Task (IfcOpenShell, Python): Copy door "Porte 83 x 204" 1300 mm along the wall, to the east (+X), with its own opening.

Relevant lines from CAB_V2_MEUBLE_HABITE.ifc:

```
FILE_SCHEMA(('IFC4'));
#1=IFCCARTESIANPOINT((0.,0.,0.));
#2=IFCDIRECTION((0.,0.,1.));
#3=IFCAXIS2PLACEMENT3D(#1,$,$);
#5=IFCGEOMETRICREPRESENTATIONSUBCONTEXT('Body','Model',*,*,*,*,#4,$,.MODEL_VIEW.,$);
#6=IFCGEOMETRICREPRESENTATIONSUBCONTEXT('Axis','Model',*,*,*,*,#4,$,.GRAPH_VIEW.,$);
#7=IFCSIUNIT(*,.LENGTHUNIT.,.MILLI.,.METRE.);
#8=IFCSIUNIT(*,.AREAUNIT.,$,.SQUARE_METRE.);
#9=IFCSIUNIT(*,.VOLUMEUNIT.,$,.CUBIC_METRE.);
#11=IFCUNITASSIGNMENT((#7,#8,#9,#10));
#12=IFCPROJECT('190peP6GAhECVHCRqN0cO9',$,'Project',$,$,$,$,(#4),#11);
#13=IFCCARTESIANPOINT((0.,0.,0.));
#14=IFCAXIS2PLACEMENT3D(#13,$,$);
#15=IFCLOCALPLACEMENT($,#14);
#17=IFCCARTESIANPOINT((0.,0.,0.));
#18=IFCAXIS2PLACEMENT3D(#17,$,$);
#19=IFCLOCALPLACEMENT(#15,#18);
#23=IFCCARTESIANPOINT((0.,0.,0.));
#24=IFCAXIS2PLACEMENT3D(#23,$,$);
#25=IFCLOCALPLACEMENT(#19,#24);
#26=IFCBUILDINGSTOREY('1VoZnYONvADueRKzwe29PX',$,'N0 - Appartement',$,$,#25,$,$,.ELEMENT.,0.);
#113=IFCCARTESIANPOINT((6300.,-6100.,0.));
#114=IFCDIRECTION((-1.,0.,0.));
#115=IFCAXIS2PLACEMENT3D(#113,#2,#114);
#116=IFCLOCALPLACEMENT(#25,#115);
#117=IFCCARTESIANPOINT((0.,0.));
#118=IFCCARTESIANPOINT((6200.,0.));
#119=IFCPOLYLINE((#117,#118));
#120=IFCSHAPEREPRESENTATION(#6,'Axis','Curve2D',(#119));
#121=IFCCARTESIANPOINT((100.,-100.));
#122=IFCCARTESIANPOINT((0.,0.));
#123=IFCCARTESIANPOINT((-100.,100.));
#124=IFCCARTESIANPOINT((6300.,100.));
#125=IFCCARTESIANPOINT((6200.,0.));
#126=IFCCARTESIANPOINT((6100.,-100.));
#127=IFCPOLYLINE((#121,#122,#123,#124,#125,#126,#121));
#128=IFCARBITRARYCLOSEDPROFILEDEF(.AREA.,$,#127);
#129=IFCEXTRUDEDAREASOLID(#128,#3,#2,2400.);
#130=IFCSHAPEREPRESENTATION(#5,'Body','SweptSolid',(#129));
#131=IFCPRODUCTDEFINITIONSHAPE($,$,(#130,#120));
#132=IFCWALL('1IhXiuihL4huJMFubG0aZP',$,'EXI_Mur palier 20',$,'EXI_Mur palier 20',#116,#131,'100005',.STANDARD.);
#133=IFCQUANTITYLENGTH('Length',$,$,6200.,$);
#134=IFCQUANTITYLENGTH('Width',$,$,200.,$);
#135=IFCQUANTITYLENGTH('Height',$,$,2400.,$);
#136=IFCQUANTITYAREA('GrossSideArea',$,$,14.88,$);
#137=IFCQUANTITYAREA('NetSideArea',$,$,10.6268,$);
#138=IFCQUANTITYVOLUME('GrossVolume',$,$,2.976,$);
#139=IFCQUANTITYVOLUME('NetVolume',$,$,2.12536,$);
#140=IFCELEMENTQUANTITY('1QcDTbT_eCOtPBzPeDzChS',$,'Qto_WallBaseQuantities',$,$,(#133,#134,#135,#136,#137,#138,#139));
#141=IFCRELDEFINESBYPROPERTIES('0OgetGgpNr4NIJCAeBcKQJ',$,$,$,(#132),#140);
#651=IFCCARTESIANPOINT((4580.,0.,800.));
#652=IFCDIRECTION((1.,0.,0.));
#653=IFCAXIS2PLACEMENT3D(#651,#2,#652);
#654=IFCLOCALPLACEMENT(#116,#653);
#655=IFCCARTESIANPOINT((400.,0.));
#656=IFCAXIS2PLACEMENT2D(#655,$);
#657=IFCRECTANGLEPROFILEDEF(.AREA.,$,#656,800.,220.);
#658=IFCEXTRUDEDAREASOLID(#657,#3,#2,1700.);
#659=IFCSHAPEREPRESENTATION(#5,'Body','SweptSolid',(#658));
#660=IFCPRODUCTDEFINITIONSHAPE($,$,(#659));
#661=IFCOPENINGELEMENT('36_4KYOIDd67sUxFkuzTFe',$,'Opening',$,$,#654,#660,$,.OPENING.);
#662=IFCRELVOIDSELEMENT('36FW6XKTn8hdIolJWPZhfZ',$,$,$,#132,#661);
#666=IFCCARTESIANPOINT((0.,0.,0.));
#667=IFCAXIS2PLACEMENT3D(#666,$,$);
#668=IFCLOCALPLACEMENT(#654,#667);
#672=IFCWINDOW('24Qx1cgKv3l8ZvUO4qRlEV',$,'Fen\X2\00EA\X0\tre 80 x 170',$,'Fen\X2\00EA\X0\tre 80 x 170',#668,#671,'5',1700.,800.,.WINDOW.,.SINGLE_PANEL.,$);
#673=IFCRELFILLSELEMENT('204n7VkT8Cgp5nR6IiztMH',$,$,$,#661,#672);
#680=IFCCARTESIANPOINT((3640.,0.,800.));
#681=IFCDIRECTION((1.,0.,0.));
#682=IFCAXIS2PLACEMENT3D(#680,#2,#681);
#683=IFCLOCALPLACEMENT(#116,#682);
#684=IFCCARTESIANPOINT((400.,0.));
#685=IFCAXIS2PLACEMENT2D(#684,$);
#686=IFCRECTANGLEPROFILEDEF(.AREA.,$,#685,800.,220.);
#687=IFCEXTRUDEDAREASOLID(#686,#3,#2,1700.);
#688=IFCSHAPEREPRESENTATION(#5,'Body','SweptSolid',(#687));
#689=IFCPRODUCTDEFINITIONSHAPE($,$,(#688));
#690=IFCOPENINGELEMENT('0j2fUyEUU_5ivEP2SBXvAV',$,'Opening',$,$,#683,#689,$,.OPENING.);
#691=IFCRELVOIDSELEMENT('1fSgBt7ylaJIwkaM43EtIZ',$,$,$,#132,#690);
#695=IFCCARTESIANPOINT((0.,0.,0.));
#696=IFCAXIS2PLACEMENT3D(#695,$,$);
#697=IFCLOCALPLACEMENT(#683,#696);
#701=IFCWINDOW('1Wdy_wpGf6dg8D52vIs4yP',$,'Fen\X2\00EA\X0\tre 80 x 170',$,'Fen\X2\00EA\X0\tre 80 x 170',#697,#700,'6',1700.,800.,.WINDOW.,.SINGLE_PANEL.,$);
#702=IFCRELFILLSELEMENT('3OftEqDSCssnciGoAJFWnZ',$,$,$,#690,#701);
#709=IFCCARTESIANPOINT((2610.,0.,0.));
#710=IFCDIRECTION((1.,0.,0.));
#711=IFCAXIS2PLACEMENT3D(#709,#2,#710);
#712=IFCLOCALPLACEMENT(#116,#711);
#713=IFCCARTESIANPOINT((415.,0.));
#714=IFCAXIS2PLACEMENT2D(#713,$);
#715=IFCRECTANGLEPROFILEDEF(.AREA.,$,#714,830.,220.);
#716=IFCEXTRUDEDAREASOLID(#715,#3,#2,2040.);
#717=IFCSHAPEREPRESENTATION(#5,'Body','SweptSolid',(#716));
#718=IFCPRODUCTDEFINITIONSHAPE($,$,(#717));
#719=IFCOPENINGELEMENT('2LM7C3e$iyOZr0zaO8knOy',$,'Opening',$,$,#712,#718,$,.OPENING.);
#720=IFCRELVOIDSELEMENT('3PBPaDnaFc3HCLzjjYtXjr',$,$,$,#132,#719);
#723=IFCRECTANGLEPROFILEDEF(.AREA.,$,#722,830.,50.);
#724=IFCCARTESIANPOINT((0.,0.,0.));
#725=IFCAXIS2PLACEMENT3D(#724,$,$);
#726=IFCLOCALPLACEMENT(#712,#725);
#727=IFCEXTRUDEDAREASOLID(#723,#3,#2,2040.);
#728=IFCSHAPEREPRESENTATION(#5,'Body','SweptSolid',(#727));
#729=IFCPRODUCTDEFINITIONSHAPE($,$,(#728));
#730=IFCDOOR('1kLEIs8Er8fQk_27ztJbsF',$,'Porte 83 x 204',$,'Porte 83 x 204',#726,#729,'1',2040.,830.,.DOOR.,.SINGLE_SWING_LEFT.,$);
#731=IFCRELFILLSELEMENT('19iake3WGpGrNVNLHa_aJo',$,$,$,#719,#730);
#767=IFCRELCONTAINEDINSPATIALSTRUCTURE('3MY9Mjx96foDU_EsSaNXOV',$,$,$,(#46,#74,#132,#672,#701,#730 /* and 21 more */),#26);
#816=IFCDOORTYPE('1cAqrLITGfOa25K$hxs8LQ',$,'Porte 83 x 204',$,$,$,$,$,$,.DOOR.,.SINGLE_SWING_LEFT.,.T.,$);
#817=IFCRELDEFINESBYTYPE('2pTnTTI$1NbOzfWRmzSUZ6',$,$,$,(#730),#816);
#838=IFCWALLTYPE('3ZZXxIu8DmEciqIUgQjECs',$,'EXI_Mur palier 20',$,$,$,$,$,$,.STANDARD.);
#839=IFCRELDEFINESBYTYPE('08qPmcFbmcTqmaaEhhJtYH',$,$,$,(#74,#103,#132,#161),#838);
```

```python
import ifcopenshell
import ifcopenshell.api.feature
import ifcopenshell.api.geometry
import ifcopenshell.api.pset
import ifcopenshell.api.root
import ifcopenshell.geom
import ifcopenshell.util.element
import ifcopenshell.util.placement
import ifcopenshell.util.shape
import ifcopenshell.util.unit

model = ifcopenshell.open("CAB_V2_MEUBLE_HABITE.ifc")
unit_scale = ifcopenshell.util.unit.calculate_unit_scale(model)
area_scale = ifcopenshell.util.unit.calculate_unit_scale(model, "AREAUNIT")
volume_scale = ifcopenshell.util.unit.calculate_unit_scale(model, "VOLUMEUNIT")
settings = ifcopenshell.geom.settings()


def volume(element):
    """Net volume in cubic metres, openings subtracted."""
    shape = ifcopenshell.geom.create_shape(settings, element)
    return ifcopenshell.util.shape.get_volume(shape.geometry)


door = model.by_guid("1kLEIs8Er8fQk_27ztJbsF")
opening = door.FillsVoids[0].RelatingOpeningElement
wall = opening.VoidsElements[0].RelatingBuildingElement
before = volume(wall)
shift = ifcopenshell.util.placement.get_local_placement(wall.ObjectPlacement)[:3, 0] * -1.3 / unit_scale

# copy_class copies the void relationship, type, container and properties, but no geometry.
new_opening = ifcopenshell.api.root.copy_class(model, product=opening)
new_opening.Representation = ifcopenshell.util.element.copy_deep(
    model, opening.Representation, exclude=["IfcGeometricRepresentationContext", "IfcRepresentationMap"]
)
new_door = ifcopenshell.api.root.copy_class(model, product=door)
new_door.Representation = ifcopenshell.util.element.copy_deep(
    model, door.Representation, exclude=["IfcGeometricRepresentationContext", "IfcRepresentationMap"]
)
new_door.Tag = None
ifcopenshell.api.feature.add_filling(model, opening=new_opening, element=new_door)

for old, new in ((opening, new_opening), (door, new_door)):
    matrix = ifcopenshell.util.placement.get_local_placement(old.ObjectPlacement)
    matrix[:3, 3] += shift
    ifcopenshell.api.geometry.edit_object_placement(model, product=new, matrix=matrix, is_si=False)

after = volume(wall)
thickness = 0.2  # wall thickness in metres

# Update the wall's stored quantities.
qto = model.by_id(ifcopenshell.util.element.get_pset(wall, "Qto_WallBaseQuantities", should_inherit=False)["id"])
ifcopenshell.api.pset.edit_qto(model, qto=qto, properties={
    "NetSideArea": after / thickness / area_scale,
    "NetVolume": after / volume_scale,
})

print(f"wall volume {before:.3f} -> {after:.3f} m3")

model.write("CAB_V2_MEUBLE_HABITE_v2.ifc")
```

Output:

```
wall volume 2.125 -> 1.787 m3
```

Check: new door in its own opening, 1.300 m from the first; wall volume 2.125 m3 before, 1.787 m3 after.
